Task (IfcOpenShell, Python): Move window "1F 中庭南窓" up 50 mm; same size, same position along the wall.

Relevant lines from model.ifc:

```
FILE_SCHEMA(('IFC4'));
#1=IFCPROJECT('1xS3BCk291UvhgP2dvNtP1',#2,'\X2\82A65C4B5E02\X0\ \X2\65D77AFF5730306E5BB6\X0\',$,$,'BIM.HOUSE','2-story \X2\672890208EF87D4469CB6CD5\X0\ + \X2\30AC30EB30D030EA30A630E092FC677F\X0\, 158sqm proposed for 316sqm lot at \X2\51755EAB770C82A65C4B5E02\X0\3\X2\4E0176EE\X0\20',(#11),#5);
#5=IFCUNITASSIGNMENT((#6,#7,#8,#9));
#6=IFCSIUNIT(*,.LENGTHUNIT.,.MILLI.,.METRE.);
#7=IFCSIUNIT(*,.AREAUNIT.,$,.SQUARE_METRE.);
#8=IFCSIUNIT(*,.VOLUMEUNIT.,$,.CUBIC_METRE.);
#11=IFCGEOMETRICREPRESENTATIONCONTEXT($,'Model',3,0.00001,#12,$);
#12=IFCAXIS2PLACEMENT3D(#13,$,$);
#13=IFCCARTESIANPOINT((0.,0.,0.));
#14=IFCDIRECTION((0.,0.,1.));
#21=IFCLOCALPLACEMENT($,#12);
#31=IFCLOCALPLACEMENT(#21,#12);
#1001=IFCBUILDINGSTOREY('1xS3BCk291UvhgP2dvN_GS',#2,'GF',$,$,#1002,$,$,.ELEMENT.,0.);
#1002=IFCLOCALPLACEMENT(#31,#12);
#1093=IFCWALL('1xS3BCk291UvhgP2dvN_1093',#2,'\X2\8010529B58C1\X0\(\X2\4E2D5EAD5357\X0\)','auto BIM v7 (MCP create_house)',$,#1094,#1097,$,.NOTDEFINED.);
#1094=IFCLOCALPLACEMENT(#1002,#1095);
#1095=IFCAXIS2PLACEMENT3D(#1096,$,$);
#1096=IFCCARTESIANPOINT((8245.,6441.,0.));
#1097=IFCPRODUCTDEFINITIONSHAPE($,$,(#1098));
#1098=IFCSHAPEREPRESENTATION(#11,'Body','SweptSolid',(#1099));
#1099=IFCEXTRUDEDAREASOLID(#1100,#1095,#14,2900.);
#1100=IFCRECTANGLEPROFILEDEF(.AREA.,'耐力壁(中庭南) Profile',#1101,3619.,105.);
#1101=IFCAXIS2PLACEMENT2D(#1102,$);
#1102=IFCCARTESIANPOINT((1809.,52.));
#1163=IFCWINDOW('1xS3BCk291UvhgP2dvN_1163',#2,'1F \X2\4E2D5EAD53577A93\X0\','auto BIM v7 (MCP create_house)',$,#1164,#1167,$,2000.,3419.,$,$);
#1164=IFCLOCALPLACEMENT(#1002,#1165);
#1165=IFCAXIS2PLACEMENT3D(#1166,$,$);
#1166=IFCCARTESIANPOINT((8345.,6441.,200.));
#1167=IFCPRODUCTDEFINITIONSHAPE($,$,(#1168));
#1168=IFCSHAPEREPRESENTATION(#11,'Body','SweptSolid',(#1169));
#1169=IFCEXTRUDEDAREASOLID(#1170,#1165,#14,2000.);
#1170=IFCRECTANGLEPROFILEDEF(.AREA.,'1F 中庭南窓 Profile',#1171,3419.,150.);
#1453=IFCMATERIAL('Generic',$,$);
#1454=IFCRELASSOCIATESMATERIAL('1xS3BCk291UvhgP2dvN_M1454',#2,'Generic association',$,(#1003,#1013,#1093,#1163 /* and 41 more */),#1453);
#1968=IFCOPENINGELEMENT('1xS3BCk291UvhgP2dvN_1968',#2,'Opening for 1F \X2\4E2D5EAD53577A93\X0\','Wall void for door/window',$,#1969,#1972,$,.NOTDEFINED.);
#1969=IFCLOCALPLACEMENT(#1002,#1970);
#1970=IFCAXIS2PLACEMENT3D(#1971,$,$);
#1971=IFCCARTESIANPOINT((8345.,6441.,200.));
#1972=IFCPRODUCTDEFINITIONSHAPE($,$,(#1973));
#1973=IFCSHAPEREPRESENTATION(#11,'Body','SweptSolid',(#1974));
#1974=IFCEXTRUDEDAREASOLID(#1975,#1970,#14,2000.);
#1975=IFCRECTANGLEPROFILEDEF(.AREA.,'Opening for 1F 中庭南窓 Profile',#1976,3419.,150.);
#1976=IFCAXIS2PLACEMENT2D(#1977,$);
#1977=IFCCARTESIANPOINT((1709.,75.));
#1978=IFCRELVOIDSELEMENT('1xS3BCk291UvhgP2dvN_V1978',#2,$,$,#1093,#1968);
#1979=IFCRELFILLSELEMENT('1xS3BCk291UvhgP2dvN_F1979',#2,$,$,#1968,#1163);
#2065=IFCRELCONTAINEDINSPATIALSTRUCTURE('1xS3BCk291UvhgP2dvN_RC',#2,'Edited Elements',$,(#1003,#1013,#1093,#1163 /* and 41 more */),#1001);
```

```python
import numpy as np
import ifcopenshell
import ifcopenshell.api.geometry
import ifcopenshell.util.placement
import ifcopenshell.util.unit

model = ifcopenshell.open("model.ifc")
unit_scale = ifcopenshell.util.unit.calculate_unit_scale(model)

window = model.by_guid("1xS3BCk291UvhgP2dvN_1163")
opening = window.FillsVoids[0].RelatingOpeningElement
dz = 50.0

shift = np.array([0.0, 0.0, dz])
# The window is not placed relative to its opening, so move both.
for product in (opening, window):
    matrix = ifcopenshell.util.placement.get_local_placement(product.ObjectPlacement)
    matrix[:3, 3] += shift
    ifcopenshell.api.geometry.edit_object_placement(model, product=product, matrix=matrix, is_si=False)

print(f"moved by {dz * unit_scale:+.3f} m")

model.write("model_updated.ifc")
```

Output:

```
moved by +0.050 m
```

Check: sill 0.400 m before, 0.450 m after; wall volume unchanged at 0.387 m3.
